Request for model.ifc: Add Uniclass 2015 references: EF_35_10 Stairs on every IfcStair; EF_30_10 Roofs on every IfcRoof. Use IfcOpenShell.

First a look at what the model holds.

```python
import ifcopenshell

model = ifcopenshell.open("model.ifc")
print(model.schema)
print("classifications:", [c.Name for c in model.by_type("IfcClassification")])
for ifc_class in ("IfcDoor", "IfcRoof", "IfcStair", "IfcWall", "IfcWindow"):
    print(ifc_class, len(model.by_type(ifc_class)))
```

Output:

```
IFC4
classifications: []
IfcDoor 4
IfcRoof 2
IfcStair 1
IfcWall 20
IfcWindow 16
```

```python
import ifcopenshell
import ifcopenshell.api.classification

model = ifcopenshell.open("model.ifc")

system = ifcopenshell.api.classification.add_classification(model, classification="Uniclass 2015")

codes = {
    "IfcStair": ("EF_35_10", "Stairs"),
    "IfcRoof": ("EF_30_10", "Roofs"),
}
for ifc_class, (code, name) in codes.items():
    products = model.by_type(ifc_class)
    ifcopenshell.api.classification.add_reference(
        model, products=products, classification=system, identification=code, name=name
    )
    print(code, len(products))

model.write("model_rev.ifc")
```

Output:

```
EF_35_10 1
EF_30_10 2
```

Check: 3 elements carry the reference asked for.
